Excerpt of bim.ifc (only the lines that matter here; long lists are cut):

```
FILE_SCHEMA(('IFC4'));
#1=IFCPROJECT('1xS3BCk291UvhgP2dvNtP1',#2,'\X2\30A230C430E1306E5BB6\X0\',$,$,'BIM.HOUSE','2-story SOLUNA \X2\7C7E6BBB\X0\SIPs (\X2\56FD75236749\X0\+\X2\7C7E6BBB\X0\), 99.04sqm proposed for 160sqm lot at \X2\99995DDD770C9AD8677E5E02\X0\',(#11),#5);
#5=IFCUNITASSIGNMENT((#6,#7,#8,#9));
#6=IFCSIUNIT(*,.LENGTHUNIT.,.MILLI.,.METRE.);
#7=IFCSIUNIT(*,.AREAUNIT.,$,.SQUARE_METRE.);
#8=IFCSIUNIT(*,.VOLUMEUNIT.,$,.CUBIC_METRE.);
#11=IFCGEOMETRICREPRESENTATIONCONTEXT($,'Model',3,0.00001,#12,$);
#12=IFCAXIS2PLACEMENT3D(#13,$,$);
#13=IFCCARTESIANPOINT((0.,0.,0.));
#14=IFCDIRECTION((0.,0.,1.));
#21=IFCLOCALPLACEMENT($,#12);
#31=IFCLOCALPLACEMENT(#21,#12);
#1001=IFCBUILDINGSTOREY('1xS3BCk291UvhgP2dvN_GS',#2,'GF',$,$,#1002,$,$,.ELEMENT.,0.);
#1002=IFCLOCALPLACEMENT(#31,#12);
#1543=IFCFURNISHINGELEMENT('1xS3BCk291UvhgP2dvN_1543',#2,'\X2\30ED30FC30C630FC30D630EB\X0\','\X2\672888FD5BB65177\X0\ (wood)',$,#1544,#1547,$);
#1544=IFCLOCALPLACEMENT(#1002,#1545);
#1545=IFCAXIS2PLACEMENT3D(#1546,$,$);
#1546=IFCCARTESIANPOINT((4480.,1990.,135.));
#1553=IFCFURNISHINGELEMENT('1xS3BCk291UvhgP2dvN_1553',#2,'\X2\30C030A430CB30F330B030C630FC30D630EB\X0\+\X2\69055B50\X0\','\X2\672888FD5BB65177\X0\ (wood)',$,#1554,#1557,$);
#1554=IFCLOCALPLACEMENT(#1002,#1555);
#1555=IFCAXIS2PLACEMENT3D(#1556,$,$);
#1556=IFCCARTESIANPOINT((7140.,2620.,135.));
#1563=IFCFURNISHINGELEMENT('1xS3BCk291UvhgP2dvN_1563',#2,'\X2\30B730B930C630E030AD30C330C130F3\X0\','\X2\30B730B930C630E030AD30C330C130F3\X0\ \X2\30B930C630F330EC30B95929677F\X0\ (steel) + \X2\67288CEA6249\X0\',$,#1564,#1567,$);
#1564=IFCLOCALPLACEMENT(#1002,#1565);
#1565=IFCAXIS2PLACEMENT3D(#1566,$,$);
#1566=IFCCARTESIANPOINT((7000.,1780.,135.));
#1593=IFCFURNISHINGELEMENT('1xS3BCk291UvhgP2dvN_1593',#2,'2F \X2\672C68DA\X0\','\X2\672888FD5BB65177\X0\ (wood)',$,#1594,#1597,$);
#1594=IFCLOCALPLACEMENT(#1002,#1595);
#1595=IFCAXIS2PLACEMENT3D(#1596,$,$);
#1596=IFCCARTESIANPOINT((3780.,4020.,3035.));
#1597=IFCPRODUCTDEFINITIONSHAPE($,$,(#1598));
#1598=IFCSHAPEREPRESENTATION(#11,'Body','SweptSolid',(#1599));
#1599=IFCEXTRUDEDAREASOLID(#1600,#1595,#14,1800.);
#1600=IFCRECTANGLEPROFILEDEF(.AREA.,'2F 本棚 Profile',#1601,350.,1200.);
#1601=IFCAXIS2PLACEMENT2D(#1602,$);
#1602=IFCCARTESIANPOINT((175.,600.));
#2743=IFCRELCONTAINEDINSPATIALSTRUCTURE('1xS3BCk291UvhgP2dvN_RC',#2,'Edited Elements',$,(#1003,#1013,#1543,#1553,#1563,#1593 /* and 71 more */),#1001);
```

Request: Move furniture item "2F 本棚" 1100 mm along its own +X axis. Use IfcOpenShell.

```python
import ifcopenshell
import ifcopenshell.api.geometry
import ifcopenshell.util.placement

model = ifcopenshell.open("bim.ifc")

item = model.by_guid("1xS3BCk291UvhgP2dvN_1593")
matrix = ifcopenshell.util.placement.get_local_placement(item.ObjectPlacement)
matrix[:3, 3] += matrix[:3, 0] * 1100.0
ifcopenshell.api.geometry.edit_object_placement(model, product=item, matrix=matrix, is_si=False)

print(ifcopenshell.util.placement.get_local_placement(item.ObjectPlacement).round(3) + 0.0)

model.write("bim-out.ifc")
```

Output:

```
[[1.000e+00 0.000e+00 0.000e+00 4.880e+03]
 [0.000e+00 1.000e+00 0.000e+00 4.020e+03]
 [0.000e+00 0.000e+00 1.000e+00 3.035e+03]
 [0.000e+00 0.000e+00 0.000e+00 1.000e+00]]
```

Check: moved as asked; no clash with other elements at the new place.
